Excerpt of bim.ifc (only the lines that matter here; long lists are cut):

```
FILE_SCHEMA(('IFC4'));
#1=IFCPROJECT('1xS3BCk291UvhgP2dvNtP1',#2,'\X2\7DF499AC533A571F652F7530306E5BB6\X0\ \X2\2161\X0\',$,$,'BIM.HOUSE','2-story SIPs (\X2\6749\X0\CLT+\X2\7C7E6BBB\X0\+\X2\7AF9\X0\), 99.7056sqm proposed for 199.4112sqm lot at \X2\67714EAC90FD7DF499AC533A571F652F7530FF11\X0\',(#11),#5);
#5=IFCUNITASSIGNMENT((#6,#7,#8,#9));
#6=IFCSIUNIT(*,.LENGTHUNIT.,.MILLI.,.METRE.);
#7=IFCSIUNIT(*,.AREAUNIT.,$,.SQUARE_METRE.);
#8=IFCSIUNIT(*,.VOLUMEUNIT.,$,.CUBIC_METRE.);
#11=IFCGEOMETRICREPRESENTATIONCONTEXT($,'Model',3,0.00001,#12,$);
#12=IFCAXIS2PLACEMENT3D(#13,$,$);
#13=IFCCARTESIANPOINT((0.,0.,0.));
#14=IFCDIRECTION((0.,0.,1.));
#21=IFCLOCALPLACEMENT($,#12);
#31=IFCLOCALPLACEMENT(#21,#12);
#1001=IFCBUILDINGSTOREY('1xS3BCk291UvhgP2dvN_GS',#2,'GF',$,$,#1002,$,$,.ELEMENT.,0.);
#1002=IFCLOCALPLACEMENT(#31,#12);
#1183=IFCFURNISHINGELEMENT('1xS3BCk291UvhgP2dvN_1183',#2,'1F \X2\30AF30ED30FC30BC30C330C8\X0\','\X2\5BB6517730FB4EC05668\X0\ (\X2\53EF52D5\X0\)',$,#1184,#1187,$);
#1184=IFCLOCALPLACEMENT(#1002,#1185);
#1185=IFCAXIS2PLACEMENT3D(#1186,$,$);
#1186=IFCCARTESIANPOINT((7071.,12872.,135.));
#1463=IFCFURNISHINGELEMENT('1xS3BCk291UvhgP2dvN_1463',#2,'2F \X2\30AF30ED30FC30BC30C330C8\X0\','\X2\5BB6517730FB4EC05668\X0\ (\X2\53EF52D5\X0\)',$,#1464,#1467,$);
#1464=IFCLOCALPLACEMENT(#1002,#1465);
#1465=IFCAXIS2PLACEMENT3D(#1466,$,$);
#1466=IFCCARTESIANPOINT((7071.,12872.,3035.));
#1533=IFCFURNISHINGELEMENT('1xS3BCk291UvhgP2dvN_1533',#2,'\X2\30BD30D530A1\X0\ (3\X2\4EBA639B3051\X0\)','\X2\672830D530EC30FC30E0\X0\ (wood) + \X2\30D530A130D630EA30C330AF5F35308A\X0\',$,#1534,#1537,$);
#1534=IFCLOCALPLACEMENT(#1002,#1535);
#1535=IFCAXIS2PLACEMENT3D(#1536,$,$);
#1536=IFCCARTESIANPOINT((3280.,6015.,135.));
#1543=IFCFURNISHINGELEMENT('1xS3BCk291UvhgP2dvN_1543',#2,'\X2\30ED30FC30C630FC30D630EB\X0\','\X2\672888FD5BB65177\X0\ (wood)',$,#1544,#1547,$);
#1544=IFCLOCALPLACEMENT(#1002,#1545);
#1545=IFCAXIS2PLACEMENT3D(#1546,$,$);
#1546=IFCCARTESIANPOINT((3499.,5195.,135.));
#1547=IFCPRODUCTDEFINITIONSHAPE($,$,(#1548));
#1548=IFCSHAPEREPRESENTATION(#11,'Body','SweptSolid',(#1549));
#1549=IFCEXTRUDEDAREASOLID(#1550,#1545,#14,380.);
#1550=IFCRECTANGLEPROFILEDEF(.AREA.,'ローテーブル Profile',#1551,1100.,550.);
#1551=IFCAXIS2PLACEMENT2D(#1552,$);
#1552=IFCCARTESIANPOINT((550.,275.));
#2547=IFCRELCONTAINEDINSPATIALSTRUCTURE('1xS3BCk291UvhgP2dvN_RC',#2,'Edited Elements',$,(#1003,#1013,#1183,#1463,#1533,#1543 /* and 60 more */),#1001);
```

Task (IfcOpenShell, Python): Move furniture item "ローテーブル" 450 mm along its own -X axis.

```python
import ifcopenshell
import ifcopenshell.api.geometry
import ifcopenshell.util.placement
import ifcopenshell.util.unit

model = ifcopenshell.open("bim.ifc")
unit_scale = ifcopenshell.util.unit.calculate_unit_scale(model)

item = model.by_guid("1xS3BCk291UvhgP2dvN_1543")
matrix = ifcopenshell.util.placement.get_local_placement(item.ObjectPlacement)
matrix[:3, 3] -= matrix[:3, 0] * 0.45 / unit_scale
ifcopenshell.api.geometry.edit_object_placement(model, product=item, matrix=matrix, is_si=False)

print(ifcopenshell.util.placement.get_local_placement(item.ObjectPlacement).round(3) + 0.0)

model.write("bim-out.ifc")
```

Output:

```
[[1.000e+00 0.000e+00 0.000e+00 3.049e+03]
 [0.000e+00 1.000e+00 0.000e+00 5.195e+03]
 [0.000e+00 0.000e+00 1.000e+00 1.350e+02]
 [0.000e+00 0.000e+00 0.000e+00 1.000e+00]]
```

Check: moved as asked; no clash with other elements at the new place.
